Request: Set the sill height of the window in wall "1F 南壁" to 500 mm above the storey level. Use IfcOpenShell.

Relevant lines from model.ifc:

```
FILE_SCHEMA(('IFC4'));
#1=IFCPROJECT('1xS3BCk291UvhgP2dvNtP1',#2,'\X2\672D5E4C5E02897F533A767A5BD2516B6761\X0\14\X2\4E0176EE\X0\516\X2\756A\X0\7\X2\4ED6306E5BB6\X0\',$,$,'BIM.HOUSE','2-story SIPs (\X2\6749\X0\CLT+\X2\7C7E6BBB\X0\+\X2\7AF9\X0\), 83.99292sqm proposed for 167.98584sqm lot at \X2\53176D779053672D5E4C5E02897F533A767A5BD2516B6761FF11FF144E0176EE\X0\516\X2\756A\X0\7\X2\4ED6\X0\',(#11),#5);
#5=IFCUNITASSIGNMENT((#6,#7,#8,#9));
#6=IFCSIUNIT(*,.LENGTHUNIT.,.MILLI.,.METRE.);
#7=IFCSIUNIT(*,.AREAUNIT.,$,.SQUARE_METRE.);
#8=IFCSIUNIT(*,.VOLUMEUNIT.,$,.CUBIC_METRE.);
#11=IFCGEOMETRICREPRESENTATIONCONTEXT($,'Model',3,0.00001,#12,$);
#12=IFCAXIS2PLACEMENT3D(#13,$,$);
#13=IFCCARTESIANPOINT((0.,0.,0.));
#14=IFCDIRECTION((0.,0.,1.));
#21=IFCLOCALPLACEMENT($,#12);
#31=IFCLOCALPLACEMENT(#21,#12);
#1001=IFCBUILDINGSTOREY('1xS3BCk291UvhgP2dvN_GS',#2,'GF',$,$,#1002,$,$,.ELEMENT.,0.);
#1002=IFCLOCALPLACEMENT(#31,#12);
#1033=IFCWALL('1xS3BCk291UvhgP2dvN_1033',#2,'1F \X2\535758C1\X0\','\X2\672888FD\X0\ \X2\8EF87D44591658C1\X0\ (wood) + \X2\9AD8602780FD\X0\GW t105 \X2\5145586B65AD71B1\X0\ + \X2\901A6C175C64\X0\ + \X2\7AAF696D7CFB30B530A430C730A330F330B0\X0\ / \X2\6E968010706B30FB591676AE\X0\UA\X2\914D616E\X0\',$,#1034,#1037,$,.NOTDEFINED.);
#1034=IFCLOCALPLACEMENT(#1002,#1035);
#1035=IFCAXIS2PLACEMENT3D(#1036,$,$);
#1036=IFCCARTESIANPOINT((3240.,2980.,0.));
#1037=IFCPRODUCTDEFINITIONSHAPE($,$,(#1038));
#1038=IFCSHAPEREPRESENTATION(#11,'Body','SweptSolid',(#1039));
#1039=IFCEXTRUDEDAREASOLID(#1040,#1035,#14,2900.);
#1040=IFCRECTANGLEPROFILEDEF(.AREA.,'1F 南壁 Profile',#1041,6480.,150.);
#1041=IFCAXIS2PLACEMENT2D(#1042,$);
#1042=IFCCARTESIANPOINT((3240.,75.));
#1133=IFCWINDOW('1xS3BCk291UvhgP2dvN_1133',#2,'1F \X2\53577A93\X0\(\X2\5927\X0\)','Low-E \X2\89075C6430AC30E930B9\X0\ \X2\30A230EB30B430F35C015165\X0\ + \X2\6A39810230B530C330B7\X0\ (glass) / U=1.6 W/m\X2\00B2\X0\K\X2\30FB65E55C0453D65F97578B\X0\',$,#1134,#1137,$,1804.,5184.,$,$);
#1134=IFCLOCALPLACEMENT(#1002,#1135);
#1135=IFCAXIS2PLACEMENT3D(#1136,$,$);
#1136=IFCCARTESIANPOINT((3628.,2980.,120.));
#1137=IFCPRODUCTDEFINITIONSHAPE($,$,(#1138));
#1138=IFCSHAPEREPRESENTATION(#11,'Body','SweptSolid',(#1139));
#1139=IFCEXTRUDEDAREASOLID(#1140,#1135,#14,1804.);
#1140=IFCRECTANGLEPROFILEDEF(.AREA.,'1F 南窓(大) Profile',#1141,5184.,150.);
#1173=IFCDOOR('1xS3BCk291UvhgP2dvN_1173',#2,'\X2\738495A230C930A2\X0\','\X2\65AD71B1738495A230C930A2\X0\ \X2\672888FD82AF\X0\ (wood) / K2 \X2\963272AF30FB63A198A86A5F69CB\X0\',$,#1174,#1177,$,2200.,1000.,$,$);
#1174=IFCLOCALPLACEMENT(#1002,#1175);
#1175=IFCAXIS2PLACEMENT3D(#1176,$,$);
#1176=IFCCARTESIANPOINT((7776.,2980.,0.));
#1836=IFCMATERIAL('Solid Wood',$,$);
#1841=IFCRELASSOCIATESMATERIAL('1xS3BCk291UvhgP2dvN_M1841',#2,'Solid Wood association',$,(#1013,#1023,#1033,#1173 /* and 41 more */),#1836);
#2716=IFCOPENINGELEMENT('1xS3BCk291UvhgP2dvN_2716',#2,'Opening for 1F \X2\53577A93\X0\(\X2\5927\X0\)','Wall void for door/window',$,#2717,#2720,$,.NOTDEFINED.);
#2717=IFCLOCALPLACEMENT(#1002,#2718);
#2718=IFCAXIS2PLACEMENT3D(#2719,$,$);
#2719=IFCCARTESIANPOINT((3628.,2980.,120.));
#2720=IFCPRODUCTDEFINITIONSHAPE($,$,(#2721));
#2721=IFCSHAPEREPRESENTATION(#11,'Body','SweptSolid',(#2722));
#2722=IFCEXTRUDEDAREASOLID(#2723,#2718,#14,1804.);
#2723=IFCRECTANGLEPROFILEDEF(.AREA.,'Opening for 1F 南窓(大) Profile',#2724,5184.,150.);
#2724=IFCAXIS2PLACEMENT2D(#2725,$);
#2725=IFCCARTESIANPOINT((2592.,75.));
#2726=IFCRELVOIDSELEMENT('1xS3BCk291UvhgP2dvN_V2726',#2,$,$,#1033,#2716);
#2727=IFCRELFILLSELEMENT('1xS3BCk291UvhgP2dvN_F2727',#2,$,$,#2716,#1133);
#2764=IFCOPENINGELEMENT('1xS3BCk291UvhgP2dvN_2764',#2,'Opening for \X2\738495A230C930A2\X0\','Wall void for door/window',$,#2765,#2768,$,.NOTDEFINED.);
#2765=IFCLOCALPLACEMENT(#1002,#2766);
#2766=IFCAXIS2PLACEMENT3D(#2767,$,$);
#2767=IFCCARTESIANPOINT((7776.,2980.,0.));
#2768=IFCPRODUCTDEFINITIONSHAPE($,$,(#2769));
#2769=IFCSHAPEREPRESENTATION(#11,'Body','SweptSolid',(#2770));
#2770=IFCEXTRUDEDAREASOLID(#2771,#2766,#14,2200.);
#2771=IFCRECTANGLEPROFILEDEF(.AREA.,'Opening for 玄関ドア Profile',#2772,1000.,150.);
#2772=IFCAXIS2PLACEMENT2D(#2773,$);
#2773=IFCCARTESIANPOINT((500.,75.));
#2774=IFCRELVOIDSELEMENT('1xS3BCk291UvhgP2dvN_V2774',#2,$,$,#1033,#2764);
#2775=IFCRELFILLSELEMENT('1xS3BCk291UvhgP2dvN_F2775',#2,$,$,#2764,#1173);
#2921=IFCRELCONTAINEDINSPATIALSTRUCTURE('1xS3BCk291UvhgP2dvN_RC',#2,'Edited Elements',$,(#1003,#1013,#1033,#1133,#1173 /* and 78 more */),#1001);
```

```python
import numpy as np
import ifcopenshell
import ifcopenshell.api.geometry
import ifcopenshell.geom
import ifcopenshell.util.element
import ifcopenshell.util.placement
import ifcopenshell.util.shape
import ifcopenshell.util.unit

model = ifcopenshell.open("model.ifc")
unit_scale = ifcopenshell.util.unit.calculate_unit_scale(model)

window = model.by_guid("1xS3BCk291UvhgP2dvN_1133")
opening = window.FillsVoids[0].RelatingOpeningElement
storey = ifcopenshell.util.element.get_container(window, ifc_class="IfcBuildingStorey")
level = ifcopenshell.util.placement.get_local_placement(storey.ObjectPlacement)[2, 3]

# The opening's origin need not be at the sill, so measure its lowest point.
shape = ifcopenshell.geom.create_shape(ifcopenshell.geom.settings(), opening)
bottom = ifcopenshell.util.shape.get_shape_bottom_elevation(shape, shape.geometry) / unit_scale
dz = level + 0.5 / unit_scale - bottom

shift = np.array([0.0, 0.0, dz])
# The window is not placed relative to its opening, so move both.
for product in (opening, window):
    matrix = ifcopenshell.util.placement.get_local_placement(product.ObjectPlacement)
    matrix[:3, 3] += shift
    ifcopenshell.api.geometry.edit_object_placement(model, product=product, matrix=matrix, is_si=False)

print(f"moved by {dz * unit_scale:+.3f} m")

model.write("model_v2.ifc")
```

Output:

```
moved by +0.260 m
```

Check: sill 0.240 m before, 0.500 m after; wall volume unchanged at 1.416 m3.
